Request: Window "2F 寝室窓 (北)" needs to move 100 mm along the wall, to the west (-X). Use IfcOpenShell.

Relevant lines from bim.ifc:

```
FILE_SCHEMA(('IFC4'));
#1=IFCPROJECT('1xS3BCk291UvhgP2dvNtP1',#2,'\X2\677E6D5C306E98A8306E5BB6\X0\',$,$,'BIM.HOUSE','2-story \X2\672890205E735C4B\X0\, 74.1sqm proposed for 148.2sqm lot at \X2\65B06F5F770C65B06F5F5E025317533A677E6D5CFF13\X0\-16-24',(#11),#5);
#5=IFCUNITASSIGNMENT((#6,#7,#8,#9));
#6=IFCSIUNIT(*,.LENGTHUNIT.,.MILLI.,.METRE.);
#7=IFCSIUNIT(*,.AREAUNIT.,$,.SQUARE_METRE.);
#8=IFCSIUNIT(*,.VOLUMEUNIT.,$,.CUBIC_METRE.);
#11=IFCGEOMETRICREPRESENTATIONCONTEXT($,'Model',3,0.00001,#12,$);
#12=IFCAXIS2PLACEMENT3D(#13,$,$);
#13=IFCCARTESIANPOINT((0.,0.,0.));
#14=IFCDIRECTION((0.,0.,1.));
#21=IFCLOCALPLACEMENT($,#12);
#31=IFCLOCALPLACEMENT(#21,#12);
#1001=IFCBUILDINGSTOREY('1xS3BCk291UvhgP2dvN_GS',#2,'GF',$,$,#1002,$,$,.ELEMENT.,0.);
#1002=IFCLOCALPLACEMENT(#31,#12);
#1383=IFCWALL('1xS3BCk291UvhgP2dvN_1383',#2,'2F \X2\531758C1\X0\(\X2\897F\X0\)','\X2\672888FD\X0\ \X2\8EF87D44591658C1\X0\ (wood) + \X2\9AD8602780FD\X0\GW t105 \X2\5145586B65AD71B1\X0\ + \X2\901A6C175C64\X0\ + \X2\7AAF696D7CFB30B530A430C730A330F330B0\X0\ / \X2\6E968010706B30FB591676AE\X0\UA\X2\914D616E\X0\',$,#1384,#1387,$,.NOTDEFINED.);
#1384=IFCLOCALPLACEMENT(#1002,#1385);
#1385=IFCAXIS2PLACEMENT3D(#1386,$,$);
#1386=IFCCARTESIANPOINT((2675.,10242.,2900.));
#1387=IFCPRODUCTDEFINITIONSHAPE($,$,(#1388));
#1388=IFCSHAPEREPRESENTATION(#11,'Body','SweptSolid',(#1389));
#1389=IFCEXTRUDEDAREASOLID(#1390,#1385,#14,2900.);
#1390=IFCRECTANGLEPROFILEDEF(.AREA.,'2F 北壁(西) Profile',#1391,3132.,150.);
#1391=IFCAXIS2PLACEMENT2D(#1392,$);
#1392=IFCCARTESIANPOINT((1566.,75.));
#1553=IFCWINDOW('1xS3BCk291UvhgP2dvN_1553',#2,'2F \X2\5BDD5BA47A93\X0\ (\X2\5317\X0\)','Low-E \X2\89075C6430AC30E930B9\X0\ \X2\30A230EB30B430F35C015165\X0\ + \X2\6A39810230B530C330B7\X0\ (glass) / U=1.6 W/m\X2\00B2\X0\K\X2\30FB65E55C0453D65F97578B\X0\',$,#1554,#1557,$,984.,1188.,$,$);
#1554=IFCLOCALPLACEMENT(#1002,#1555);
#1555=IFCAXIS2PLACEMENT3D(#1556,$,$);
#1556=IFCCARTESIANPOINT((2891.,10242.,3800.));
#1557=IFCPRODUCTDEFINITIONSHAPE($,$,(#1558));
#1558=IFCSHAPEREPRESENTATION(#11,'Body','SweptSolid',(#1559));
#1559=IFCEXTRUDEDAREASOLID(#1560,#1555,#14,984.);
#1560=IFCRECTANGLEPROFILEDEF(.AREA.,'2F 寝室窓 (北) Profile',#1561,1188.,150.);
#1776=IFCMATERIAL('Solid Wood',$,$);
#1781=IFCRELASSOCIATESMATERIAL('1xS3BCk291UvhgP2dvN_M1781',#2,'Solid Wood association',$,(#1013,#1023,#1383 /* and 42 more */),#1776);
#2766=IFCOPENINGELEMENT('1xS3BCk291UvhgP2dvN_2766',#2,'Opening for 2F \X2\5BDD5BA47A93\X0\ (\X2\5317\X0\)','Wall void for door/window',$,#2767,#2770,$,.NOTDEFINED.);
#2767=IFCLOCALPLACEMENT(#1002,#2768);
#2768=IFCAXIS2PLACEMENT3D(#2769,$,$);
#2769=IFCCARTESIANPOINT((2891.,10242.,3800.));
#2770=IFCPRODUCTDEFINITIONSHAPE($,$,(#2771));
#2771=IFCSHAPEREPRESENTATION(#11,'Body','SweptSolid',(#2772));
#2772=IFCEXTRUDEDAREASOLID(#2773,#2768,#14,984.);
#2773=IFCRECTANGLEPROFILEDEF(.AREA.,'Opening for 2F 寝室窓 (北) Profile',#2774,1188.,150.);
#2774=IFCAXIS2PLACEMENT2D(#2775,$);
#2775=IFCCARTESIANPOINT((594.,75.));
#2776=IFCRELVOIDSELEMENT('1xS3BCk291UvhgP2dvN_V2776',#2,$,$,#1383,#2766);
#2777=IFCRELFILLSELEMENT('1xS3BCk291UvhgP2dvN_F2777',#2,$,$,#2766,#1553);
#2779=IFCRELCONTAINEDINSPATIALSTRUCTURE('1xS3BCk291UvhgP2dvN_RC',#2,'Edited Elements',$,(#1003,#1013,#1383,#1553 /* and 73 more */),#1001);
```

```python
import ifcopenshell
import ifcopenshell.api.geometry
import ifcopenshell.util.placement
import ifcopenshell.util.unit

model = ifcopenshell.open("bim.ifc")
unit_scale = ifcopenshell.util.unit.calculate_unit_scale(model)

window = model.by_guid("1xS3BCk291UvhgP2dvN_1553")
opening = window.FillsVoids[0].RelatingOpeningElement
wall = opening.VoidsElements[0].RelatingBuildingElement

wall_matrix = ifcopenshell.util.placement.get_local_placement(wall.ObjectPlacement)
shift = wall_matrix[:3, 0] * -0.1 / unit_scale
before = ifcopenshell.util.placement.get_local_placement(window.ObjectPlacement)[:3, 3].copy()

# The window is not placed relative to its opening, so move both.
for product in (opening, window):
    matrix = ifcopenshell.util.placement.get_local_placement(product.ObjectPlacement)
    matrix[:3, 3] += shift
    ifcopenshell.api.geometry.edit_object_placement(model, product=product, matrix=matrix, is_si=False)

after = ifcopenshell.util.placement.get_local_placement(window.ObjectPlacement)[:3, 3]
print("window moved by", (after - before).round(3) + 0.0)

model.write("bim_updated.ifc")
```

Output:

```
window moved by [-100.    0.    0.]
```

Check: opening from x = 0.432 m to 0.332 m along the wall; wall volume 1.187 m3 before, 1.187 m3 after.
